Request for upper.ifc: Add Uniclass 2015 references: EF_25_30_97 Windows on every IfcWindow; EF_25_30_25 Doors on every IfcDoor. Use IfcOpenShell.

First a look at what the model holds.

```python
import ifcopenshell

model = ifcopenshell.open("upper.ifc")
print(model.schema)
print("classifications:", [c.Name for c in model.by_type("IfcClassification")])
for ifc_class in ("IfcDoor", "IfcRoof", "IfcStair", "IfcWall", "IfcWindow"):
    print(ifc_class, len(model.by_type(ifc_class)))
```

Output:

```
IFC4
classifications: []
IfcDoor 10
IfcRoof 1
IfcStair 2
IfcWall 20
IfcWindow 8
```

```python
import ifcopenshell
import ifcopenshell.api.classification

model = ifcopenshell.open("upper.ifc")

system = ifcopenshell.api.classification.add_classification(model, classification="Uniclass 2015")

codes = {
    "IfcWindow": ("EF_25_30_97", "Windows"),
    "IfcDoor": ("EF_25_30_25", "Doors"),
}
for ifc_class, (code, name) in codes.items():
    products = model.by_type(ifc_class)
    ifcopenshell.api.classification.add_reference(
        model, products=products, classification=system, identification=code, name=name
    )
    print(code, len(products))

model.write("upper_edited.ifc")
```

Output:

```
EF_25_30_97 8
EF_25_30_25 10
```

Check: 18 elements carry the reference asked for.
